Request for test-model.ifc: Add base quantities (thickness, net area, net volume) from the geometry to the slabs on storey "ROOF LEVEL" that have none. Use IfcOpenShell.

First a look at what the model holds.

```python
import ifcopenshell
import ifcopenshell.util.element
import ifcopenshell.util.unit

model = ifcopenshell.open("test-model.ifc")
print(model.schema)
for unit_type in ("LENGTHUNIT", "AREAUNIT", "VOLUMEUNIT"):
    print(unit_type, ifcopenshell.util.unit.calculate_unit_scale(model, unit_type))
storey = next(s for s in model.by_type("IfcBuildingStorey") if s.Name == "ROOF LEVEL")
slabs = [e for e in ifcopenshell.util.element.get_decomposition(storey) if e.is_a("IfcSlab")]
for e in sorted(slabs, key=lambda e: e.id()):
    print(e.id(), e.is_a(), e.Name, list(ifcopenshell.util.element.get_psets(e, qtos_only=True)), sep=" | ")
```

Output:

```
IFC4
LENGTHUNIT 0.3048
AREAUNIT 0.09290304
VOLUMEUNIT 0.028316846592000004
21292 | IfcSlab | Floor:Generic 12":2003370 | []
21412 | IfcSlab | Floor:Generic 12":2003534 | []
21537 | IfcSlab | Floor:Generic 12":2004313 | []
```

```python
import ifcopenshell
import ifcopenshell.api.pset
import ifcopenshell.geom
import ifcopenshell.util.element
import ifcopenshell.util.shape
import ifcopenshell.util.unit

model = ifcopenshell.open("test-model.ifc")
unit_scale = ifcopenshell.util.unit.calculate_unit_scale(model)
area_scale = ifcopenshell.util.unit.calculate_unit_scale(model, "AREAUNIT")
volume_scale = ifcopenshell.util.unit.calculate_unit_scale(model, "VOLUMEUNIT")
settings = ifcopenshell.geom.settings()

storey = next(s for s in model.by_type("IfcBuildingStorey") if s.Name == "ROOF LEVEL")
slabs = [e for e in ifcopenshell.util.element.get_decomposition(storey) if e.is_a("IfcSlab")]

for e in sorted(slabs, key=lambda e: e.id()):
    if ifcopenshell.util.element.get_psets(e, qtos_only=True, should_inherit=False):
        continue
    # Geometry comes back in metres, in the element's own axes.
    shape = ifcopenshell.geom.create_shape(settings, e)
    values = {
        "Width": ifcopenshell.util.shape.get_z(shape.geometry) / unit_scale,
        "NetArea": ifcopenshell.util.shape.get_footprint_area(shape.geometry) / area_scale,
        "NetVolume": ifcopenshell.util.shape.get_volume(shape.geometry) / volume_scale,
    }
    qto = ifcopenshell.api.pset.add_qto(model, product=e, name="Qto_SlabBaseQuantities")
    ifcopenshell.api.pset.edit_qto(model, qto=qto, properties=values)
    print(e.id(), {k: round(v, 3) for k, v in values.items()})

model.write("test-model-out.ifc")
```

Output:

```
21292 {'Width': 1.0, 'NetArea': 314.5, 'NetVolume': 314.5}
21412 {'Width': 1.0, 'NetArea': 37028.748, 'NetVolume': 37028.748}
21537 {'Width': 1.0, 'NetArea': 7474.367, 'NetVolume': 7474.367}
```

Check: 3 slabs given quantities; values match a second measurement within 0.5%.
